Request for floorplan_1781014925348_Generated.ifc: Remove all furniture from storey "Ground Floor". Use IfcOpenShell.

First a look at what the model holds.

```python
import ifcopenshell
import ifcopenshell.util.element

model = ifcopenshell.open("floorplan_1781014925348_Generated.ifc")
print(model.schema)
storey = next(s for s in model.by_type("IfcBuildingStorey") if s.Name == "Ground Floor")
furniture = [e for e in ifcopenshell.util.element.get_decomposition(storey) if e.is_a("IfcFurnishingElement")]
seen = {}
for e in furniture:
    element_type = ifcopenshell.util.element.get_type(e)
    name = element_type.Name if element_type not in (None, e) else None
    seen[name] = seen.get(name, 0) + 1
for name, count in sorted(seen.items(), key=str):
    print(count, "x", name)
```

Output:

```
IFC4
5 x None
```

```python
import ifcopenshell
import ifcopenshell.api.root
import ifcopenshell.util.element

model = ifcopenshell.open("floorplan_1781014925348_Generated.ifc")

storey = next(s for s in model.by_type("IfcBuildingStorey") if s.Name == "Ground Floor")
furniture = [e for e in ifcopenshell.util.element.get_decomposition(storey) if e.is_a("IfcFurnishingElement")]

for e in furniture:
    ifcopenshell.api.root.remove_product(model, product=e)
print(len(furniture), "removed")

model.write("floorplan_1781014925348_Generated_edited.ifc")
```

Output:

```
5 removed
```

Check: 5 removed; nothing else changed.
